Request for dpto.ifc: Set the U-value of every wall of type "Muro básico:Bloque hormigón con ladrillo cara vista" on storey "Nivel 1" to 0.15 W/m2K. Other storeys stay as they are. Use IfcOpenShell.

First a look at what the model holds.

```python
import ifcopenshell
import ifcopenshell.util.element

model = ifcopenshell.open("dpto.ifc")
print(model.schema)
storey = next(s for s in model.by_type("IfcBuildingStorey") if s.Name == "Nivel 1")
walls = [e for e in ifcopenshell.util.element.get_decomposition(storey) if e.is_a("IfcWall")]
seen = {}
for e in walls:
    element_type = ifcopenshell.util.element.get_type(e)
    key = (element_type.Name if element_type != e and element_type else None, ifcopenshell.util.element.get_pset(e, "Pset_WallCommon", "ThermalTransmittance"))
    seen[key] = seen.get(key, 0) + 1
for (name, value), count in sorted(seen.items(), key=str):
    print(count, "x", name, "|", value)
```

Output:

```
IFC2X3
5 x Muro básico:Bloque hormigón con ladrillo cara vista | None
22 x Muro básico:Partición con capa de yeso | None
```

```python
import ifcopenshell
import ifcopenshell.api.pset
import ifcopenshell.util.element

model = ifcopenshell.open("dpto.ifc")

storey = next(s for s in model.by_type("IfcBuildingStorey") if s.Name == "Nivel 1")
walls = [e for e in ifcopenshell.util.element.get_decomposition(storey) if e.is_a("IfcWall")]

count = 0
for e in walls:
    element_type = ifcopenshell.util.element.get_type(e)
    if element_type in (None, e) or element_type.Name != "Muro básico:Bloque hormigón con ladrillo cara vista":
        continue
    # add_pset returns the element's existing set when there is one.
    pset = ifcopenshell.api.pset.add_pset(model, product=e, name="Pset_WallCommon")
    ifcopenshell.api.pset.edit_pset(model, pset=pset, properties={"ThermalTransmittance": 0.15})
    count += 1

print(count, "walls updated")

model.write("dpto_v2.ifc")
```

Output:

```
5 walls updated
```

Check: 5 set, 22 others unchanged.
